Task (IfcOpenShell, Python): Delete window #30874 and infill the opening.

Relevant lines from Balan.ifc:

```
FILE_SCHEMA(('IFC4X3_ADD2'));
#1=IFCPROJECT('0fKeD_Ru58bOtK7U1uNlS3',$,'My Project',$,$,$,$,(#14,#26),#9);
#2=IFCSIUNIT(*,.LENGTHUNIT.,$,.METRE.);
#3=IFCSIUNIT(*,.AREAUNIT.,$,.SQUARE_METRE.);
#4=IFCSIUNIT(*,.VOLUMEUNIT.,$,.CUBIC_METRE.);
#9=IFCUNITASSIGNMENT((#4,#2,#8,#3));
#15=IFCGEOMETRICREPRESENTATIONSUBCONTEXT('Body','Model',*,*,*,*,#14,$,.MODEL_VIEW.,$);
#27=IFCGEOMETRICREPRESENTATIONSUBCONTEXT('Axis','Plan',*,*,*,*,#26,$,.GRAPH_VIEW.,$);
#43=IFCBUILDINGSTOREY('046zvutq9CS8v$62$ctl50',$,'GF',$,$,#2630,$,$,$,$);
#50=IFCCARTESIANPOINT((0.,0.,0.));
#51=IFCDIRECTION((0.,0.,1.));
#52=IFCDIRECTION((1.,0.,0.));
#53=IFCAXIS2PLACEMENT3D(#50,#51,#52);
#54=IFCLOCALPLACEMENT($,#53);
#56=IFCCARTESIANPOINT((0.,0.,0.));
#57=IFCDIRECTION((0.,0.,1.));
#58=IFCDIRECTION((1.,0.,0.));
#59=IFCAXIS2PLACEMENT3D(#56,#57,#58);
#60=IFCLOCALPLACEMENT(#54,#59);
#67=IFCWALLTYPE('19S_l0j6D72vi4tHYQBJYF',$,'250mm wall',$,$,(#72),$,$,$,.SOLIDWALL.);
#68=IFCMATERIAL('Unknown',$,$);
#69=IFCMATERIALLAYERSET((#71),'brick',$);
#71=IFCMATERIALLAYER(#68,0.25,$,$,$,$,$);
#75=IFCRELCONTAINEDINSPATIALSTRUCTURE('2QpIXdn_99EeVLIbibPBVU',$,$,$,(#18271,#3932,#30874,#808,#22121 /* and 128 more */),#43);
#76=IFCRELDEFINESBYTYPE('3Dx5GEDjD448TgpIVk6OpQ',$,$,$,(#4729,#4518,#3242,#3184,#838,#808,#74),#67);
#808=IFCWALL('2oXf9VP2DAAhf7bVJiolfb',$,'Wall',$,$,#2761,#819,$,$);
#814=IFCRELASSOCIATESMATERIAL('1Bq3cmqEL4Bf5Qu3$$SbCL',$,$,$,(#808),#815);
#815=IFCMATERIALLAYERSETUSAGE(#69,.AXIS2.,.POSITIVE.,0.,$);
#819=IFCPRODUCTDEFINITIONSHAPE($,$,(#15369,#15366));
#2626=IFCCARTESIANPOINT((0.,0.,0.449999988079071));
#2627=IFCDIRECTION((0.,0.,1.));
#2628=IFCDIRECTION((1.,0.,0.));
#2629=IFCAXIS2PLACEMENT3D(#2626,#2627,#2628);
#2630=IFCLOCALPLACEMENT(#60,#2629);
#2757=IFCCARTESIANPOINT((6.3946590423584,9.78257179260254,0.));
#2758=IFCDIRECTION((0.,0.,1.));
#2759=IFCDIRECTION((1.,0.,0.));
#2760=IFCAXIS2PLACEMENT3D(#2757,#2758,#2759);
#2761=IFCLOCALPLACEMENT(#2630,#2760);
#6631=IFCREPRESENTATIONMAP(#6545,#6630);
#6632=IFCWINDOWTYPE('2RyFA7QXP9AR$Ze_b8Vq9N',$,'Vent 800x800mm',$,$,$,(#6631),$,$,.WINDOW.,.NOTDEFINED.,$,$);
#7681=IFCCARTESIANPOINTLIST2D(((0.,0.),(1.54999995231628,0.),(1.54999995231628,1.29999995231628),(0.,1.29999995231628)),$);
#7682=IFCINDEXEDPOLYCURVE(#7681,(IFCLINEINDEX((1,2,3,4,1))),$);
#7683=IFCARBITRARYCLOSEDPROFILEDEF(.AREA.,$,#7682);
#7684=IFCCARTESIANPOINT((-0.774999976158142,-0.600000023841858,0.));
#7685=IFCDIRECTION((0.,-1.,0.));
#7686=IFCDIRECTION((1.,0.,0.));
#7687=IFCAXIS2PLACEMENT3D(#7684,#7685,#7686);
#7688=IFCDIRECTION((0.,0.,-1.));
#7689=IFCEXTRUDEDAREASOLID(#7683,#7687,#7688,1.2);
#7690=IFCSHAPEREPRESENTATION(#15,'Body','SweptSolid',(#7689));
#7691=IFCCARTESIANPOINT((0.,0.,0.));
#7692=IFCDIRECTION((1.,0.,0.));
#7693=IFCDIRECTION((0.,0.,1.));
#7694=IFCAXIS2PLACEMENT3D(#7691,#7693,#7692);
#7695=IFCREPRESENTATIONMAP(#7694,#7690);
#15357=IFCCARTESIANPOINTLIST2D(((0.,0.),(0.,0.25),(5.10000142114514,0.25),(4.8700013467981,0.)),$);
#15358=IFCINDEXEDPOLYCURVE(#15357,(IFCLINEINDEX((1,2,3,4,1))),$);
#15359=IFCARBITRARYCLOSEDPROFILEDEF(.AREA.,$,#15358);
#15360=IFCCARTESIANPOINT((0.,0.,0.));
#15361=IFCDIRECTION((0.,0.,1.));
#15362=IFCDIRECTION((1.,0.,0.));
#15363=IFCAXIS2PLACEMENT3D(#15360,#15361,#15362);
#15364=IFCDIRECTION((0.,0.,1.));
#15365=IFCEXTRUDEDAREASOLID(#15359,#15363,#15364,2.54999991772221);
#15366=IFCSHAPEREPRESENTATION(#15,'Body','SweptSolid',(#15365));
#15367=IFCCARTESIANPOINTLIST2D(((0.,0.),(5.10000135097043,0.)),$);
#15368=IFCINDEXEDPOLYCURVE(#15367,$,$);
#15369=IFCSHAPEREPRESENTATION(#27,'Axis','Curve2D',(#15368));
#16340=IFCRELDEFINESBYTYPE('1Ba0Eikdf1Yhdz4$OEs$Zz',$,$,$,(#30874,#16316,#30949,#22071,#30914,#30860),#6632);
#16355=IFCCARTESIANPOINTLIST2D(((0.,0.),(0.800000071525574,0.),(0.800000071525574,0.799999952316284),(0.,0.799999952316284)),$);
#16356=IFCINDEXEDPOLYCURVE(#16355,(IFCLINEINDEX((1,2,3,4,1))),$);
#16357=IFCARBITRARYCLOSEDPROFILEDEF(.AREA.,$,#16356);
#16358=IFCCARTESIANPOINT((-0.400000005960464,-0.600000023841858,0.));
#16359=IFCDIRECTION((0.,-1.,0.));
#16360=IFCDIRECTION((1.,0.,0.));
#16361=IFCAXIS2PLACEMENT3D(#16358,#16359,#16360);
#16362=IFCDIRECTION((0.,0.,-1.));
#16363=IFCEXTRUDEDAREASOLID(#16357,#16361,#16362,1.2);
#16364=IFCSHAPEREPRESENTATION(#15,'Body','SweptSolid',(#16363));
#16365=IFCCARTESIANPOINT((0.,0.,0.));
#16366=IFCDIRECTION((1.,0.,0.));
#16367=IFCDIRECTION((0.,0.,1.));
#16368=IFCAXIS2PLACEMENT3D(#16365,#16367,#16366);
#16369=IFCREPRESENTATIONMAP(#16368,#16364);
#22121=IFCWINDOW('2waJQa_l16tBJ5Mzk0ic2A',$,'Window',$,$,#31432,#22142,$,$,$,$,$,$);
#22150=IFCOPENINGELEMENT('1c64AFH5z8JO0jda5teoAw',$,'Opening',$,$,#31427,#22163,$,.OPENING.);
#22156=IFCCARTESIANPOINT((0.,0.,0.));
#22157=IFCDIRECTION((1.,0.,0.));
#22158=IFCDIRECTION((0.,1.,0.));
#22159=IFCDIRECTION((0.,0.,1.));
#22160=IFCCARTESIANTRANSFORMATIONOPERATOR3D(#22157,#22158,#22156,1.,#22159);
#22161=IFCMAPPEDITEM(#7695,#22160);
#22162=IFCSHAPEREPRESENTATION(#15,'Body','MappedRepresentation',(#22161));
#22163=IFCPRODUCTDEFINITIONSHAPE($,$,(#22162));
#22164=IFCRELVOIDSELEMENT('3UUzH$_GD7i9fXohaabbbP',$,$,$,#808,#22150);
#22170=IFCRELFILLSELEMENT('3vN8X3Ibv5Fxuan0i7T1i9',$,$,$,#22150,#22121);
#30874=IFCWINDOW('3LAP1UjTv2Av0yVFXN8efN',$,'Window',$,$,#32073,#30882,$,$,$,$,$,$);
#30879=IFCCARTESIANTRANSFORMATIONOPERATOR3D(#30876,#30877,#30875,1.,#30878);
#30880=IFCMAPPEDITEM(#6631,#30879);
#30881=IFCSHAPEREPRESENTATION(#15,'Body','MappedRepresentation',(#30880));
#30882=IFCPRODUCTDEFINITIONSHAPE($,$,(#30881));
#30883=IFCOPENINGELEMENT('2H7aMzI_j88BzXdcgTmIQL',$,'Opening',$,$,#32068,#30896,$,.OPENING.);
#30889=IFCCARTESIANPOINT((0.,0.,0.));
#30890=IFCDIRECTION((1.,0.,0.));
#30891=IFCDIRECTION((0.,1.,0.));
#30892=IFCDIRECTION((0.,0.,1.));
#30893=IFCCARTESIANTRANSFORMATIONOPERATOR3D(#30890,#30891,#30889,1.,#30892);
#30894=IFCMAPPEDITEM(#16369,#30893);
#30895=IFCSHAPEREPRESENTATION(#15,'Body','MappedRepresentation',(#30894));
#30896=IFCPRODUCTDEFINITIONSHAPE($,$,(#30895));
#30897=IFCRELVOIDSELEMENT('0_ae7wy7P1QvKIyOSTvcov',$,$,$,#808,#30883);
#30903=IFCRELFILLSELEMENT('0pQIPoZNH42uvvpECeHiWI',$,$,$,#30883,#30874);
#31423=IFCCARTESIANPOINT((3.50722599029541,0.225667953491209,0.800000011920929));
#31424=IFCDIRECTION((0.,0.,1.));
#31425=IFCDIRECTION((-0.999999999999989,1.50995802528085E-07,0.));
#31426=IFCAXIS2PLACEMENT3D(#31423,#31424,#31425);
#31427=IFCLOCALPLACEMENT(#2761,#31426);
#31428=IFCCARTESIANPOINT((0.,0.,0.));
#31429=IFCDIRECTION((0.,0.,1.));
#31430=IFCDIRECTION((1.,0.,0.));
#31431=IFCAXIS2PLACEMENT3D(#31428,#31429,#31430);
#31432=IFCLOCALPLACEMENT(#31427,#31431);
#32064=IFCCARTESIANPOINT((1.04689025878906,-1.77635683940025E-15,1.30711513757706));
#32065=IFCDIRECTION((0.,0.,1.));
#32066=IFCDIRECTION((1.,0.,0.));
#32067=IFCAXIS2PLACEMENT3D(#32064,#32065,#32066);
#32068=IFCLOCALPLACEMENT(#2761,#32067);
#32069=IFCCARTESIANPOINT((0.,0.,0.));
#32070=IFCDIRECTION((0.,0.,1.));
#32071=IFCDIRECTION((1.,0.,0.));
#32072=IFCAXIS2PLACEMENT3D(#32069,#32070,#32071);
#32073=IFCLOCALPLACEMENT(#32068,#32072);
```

```python
import ifcopenshell
import ifcopenshell.api.feature
import ifcopenshell.api.root
import ifcopenshell.geom
import ifcopenshell.util.shape

model = ifcopenshell.open("Balan.ifc")
settings = ifcopenshell.geom.settings()


def volume(element):
    """Net volume in cubic metres, openings subtracted."""
    shape = ifcopenshell.geom.create_shape(settings, element)
    return ifcopenshell.util.shape.get_volume(shape.geometry)


window = model.by_guid("3LAP1UjTv2Av0yVFXN8efN")
opening = window.FillsVoids[0].RelatingOpeningElement
wall = opening.VoidsElements[0].RelatingBuildingElement
before = volume(wall)

ifcopenshell.api.root.remove_product(model, product=window)
ifcopenshell.api.feature.remove_feature(model, feature=opening)

after = volume(wall)

print(f"wall volume {before:.3f} -> {after:.3f} m3")

model.write("Balan-out.ifc")
```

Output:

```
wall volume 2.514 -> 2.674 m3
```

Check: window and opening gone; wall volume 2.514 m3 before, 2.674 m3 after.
